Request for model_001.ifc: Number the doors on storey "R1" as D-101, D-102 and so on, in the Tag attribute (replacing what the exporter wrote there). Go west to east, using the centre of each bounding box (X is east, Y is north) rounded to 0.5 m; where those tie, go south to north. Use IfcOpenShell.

First a look at what the model holds.

```python
import ifcopenshell
import ifcopenshell.util.element
import ifcopenshell.util.placement

model = ifcopenshell.open("model_001.ifc")
print(model.schema)
storey = next(s for s in model.by_type("IfcBuildingStorey") if s.Name == "R1")
doors = [e for e in ifcopenshell.util.element.get_decomposition(storey) if e.is_a("IfcDoor")]
for e in sorted(doors, key=lambda e: e.id()):
    origin = ifcopenshell.util.placement.get_local_placement(e.ObjectPlacement)[:3, 3]
    print(e.id(), e.Tag, e.Name, origin.round(2) + 0.0, sep=" | ")
```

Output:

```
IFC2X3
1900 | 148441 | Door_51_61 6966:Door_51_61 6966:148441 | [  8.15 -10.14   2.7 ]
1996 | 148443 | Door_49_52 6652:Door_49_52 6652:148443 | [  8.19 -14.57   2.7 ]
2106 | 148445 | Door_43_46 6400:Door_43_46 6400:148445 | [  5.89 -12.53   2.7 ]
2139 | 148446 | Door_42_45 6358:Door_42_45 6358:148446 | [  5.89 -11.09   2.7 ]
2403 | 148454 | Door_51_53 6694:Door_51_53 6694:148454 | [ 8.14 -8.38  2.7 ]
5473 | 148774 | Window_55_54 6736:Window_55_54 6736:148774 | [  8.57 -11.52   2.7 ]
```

```python
import ifcopenshell
import ifcopenshell.geom
import ifcopenshell.util.element
import ifcopenshell.util.shape

model = ifcopenshell.open("model_001.ifc")
settings = ifcopenshell.geom.settings()
settings.set("use-world-coords", True)


def centre(element):
    shape = ifcopenshell.geom.create_shape(settings, element)
    return ifcopenshell.util.shape.get_bbox_centroid(shape.geometry)


storey = next(s for s in model.by_type("IfcBuildingStorey") if s.Name == "R1")
doors = [e for e in ifcopenshell.util.element.get_decomposition(storey) if e.is_a("IfcDoor")]

# Insertion points can sit at a corner or the storey origin, so sort by the geometry (in metres).
centres = {e: centre(e) for e in doors}
doors.sort(key=lambda e: (round(centres[e][0] / 0.5), centres[e][1]))

for i, e in enumerate(doors, start=1):
    number = f"D-1{i:02d}"
    e.Tag = number
    print(e.id(), number)

model.write("model_001_v2.ifc")
```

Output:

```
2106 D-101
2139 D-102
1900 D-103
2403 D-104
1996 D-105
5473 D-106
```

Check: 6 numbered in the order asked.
